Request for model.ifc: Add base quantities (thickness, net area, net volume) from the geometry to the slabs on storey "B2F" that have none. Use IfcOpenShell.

First a look at what the model holds.

```python
import ifcopenshell
import ifcopenshell.util.element
import ifcopenshell.util.unit

model = ifcopenshell.open("model.ifc")
print(model.schema)
for unit_type in ("LENGTHUNIT", "AREAUNIT", "VOLUMEUNIT"):
    print(unit_type, ifcopenshell.util.unit.calculate_unit_scale(model, unit_type))
storey = next(s for s in model.by_type("IfcBuildingStorey") if s.Name == "B2F")
slabs = [e for e in ifcopenshell.util.element.get_decomposition(storey) if e.is_a("IfcSlab")]
for e in sorted(slabs, key=lambda e: e.id()):
    print(e.id(), e.is_a(), e.Name, list(ifcopenshell.util.element.get_psets(e, qtos_only=True)), sep=" | ")
```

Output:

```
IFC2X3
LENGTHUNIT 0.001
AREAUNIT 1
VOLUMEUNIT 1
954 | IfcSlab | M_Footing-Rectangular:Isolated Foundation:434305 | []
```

```python
import ifcopenshell
import ifcopenshell.api.pset
import ifcopenshell.geom
import ifcopenshell.util.element
import ifcopenshell.util.shape
import ifcopenshell.util.unit

model = ifcopenshell.open("model.ifc")
unit_scale = ifcopenshell.util.unit.calculate_unit_scale(model)
area_scale = ifcopenshell.util.unit.calculate_unit_scale(model, "AREAUNIT")
volume_scale = ifcopenshell.util.unit.calculate_unit_scale(model, "VOLUMEUNIT")
settings = ifcopenshell.geom.settings()

storey = next(s for s in model.by_type("IfcBuildingStorey") if s.Name == "B2F")
slabs = [e for e in ifcopenshell.util.element.get_decomposition(storey) if e.is_a("IfcSlab")]

for e in sorted(slabs, key=lambda e: e.id()):
    if ifcopenshell.util.element.get_psets(e, qtos_only=True, should_inherit=False):
        continue
    # Geometry comes back in metres, in the element's own axes.
    shape = ifcopenshell.geom.create_shape(settings, e)
    values = {
        "Width": ifcopenshell.util.shape.get_z(shape.geometry) / unit_scale,
        "NetArea": ifcopenshell.util.shape.get_footprint_area(shape.geometry) / area_scale,
        "NetVolume": ifcopenshell.util.shape.get_volume(shape.geometry) / volume_scale,
    }
    qto = ifcopenshell.api.pset.add_qto(model, product=e, name="BaseQuantities")
    ifcopenshell.api.pset.edit_qto(model, qto=qto, properties=values)
    print(e.id(), {k: round(v, 3) for k, v in values.items()})

model.write("model_edited.ifc")
```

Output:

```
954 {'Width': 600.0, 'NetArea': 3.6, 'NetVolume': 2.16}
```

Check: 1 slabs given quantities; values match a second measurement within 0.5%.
